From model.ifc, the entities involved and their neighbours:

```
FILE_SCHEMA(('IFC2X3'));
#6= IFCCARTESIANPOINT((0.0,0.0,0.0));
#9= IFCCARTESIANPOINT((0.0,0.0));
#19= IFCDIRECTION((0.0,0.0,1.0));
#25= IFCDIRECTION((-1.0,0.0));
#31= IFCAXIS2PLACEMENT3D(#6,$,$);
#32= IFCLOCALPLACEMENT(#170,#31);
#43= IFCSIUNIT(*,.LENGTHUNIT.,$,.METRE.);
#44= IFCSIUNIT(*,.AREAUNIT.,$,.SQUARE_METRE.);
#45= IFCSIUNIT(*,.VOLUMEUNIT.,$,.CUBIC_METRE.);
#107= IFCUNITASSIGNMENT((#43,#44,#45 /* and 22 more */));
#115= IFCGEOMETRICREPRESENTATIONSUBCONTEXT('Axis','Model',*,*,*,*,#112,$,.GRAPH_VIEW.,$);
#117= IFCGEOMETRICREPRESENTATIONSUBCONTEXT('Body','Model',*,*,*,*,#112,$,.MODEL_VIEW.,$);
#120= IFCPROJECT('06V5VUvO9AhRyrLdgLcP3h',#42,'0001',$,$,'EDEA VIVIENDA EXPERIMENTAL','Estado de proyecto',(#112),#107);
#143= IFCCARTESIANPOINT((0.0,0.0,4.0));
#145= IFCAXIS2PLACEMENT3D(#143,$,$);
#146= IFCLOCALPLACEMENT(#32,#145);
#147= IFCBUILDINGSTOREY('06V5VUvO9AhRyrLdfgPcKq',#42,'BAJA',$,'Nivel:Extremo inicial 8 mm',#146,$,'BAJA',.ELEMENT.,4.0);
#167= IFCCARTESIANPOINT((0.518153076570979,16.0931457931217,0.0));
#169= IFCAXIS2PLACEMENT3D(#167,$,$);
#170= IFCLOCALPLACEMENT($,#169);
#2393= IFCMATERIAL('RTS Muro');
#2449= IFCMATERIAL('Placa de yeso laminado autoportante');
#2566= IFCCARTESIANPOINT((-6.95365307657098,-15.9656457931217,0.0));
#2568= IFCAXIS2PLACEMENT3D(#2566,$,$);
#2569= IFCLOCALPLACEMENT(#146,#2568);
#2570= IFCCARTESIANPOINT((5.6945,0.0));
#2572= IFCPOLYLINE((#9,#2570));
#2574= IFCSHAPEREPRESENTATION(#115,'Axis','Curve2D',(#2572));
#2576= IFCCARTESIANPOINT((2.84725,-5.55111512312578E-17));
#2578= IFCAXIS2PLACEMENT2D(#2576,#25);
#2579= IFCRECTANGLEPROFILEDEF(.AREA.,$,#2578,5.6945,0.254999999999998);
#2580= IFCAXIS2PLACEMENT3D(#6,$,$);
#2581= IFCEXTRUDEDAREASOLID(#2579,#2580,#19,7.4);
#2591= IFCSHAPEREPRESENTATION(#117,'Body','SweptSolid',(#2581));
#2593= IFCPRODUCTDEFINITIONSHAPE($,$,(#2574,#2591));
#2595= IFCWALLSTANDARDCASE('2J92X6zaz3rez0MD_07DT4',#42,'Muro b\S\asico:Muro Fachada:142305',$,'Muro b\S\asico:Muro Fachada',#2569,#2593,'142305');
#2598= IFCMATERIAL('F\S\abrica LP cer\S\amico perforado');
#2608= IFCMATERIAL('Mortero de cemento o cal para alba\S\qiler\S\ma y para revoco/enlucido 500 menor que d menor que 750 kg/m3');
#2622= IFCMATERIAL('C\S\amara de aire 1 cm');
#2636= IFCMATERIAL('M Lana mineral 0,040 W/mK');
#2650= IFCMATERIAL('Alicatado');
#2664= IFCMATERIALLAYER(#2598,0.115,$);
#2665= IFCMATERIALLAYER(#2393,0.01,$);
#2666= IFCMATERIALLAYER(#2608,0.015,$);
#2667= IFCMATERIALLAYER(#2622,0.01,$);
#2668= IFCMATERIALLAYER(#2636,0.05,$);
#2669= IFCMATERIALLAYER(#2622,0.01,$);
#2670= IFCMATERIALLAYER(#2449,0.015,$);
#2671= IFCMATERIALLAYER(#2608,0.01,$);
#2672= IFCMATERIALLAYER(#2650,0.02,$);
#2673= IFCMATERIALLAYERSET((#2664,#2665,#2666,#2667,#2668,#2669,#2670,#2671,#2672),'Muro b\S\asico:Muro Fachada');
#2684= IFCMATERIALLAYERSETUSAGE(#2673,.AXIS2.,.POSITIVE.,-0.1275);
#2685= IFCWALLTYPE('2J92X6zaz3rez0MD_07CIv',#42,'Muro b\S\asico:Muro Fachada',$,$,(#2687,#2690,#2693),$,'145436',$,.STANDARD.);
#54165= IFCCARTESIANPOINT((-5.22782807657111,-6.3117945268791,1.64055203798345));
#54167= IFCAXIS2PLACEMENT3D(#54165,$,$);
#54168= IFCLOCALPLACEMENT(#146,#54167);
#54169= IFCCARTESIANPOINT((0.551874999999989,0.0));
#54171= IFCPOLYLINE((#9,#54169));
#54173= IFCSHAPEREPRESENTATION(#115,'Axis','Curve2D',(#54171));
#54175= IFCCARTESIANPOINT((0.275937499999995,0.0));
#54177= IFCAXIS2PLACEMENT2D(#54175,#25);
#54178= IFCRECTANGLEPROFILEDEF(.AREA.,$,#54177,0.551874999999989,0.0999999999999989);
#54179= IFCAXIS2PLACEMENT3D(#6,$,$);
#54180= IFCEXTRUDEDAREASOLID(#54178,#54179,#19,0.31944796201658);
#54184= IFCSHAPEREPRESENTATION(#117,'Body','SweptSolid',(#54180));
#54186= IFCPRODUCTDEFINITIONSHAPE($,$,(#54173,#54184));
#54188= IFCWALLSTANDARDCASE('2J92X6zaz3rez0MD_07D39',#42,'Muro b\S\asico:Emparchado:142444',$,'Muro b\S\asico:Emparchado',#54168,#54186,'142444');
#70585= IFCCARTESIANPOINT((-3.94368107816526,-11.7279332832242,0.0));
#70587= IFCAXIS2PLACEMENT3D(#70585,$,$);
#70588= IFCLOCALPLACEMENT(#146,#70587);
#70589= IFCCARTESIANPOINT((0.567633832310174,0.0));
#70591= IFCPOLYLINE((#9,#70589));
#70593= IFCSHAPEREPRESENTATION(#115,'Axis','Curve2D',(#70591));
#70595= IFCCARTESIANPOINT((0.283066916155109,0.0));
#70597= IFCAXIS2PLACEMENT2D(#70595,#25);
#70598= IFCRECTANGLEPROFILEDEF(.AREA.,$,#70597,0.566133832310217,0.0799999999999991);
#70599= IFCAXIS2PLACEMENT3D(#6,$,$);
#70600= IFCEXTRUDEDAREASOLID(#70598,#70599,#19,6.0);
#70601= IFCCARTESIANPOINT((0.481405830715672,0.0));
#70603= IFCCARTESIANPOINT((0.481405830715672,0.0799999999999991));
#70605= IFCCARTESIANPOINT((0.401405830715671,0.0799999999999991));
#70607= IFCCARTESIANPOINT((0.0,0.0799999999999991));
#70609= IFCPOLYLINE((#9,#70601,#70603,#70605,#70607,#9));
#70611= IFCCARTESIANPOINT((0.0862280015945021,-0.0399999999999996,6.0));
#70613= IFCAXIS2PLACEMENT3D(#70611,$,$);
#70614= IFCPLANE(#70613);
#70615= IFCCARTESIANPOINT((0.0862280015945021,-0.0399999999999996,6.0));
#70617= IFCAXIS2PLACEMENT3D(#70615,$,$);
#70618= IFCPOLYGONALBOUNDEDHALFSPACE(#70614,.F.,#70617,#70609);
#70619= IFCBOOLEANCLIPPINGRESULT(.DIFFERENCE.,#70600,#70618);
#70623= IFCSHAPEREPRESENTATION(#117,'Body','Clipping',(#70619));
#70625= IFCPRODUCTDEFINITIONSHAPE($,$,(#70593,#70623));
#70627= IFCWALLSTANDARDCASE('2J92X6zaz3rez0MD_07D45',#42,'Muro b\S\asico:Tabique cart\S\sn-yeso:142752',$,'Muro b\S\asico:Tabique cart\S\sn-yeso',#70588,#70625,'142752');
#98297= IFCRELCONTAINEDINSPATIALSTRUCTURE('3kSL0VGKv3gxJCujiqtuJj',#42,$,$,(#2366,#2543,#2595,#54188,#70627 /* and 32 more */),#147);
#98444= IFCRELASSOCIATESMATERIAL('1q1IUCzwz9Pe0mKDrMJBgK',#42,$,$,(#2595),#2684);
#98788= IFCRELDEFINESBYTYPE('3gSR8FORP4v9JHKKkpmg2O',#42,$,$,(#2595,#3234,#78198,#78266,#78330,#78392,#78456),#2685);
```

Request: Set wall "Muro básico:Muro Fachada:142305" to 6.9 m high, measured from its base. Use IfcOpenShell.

```python
import ifcopenshell
import ifcopenshell.geom
import ifcopenshell.util.representation
import ifcopenshell.util.shape
import ifcopenshell.util.unit

model = ifcopenshell.open("model.ifc")
unit_scale = ifcopenshell.util.unit.calculate_unit_scale(model)
settings = ifcopenshell.geom.settings()


def volume(element):
    """Net volume in cubic metres, openings subtracted."""
    shape = ifcopenshell.geom.create_shape(settings, element)
    return ifcopenshell.util.shape.get_volume(shape.geometry)


wall = model.by_guid("2J92X6zaz3rez0MD_07DT4")
before = volume(wall)

body = ifcopenshell.util.representation.get_representation(wall, "Model", "Body")
solid = body.Items[0]
old_height = solid.Depth
solid.Depth = 6.9 / unit_scale
after = volume(wall)

print(f"height {old_height:g} -> {solid.Depth:g}, volume {before:.3f} -> {after:.3f} m3")

model.write("model_edited.ifc")
```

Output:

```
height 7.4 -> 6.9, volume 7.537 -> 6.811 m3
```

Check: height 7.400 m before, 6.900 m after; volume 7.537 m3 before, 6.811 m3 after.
